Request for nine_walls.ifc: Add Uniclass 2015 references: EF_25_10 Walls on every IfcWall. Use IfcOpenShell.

First a look at what the model holds.

```python
import ifcopenshell

model = ifcopenshell.open("nine_walls.ifc")
print(model.schema)
print("classifications:", [c.Name for c in model.by_type("IfcClassification")])
for ifc_class in ("IfcDoor", "IfcRoof", "IfcStair", "IfcWall", "IfcWindow"):
    print(ifc_class, len(model.by_type(ifc_class)))
```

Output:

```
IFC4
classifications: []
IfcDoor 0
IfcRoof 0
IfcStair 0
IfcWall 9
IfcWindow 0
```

```python
import ifcopenshell
import ifcopenshell.api.classification

model = ifcopenshell.open("nine_walls.ifc")

system = ifcopenshell.api.classification.add_classification(model, classification="Uniclass 2015")

codes = {
    "IfcWall": ("EF_25_10", "Walls"),
}
for ifc_class, (code, name) in codes.items():
    products = model.by_type(ifc_class)
    ifcopenshell.api.classification.add_reference(
        model, products=products, classification=system, identification=code, name=name
    )
    print(code, len(products))

model.write("nine_walls_edited.ifc")
```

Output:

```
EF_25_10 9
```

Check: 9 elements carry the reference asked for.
